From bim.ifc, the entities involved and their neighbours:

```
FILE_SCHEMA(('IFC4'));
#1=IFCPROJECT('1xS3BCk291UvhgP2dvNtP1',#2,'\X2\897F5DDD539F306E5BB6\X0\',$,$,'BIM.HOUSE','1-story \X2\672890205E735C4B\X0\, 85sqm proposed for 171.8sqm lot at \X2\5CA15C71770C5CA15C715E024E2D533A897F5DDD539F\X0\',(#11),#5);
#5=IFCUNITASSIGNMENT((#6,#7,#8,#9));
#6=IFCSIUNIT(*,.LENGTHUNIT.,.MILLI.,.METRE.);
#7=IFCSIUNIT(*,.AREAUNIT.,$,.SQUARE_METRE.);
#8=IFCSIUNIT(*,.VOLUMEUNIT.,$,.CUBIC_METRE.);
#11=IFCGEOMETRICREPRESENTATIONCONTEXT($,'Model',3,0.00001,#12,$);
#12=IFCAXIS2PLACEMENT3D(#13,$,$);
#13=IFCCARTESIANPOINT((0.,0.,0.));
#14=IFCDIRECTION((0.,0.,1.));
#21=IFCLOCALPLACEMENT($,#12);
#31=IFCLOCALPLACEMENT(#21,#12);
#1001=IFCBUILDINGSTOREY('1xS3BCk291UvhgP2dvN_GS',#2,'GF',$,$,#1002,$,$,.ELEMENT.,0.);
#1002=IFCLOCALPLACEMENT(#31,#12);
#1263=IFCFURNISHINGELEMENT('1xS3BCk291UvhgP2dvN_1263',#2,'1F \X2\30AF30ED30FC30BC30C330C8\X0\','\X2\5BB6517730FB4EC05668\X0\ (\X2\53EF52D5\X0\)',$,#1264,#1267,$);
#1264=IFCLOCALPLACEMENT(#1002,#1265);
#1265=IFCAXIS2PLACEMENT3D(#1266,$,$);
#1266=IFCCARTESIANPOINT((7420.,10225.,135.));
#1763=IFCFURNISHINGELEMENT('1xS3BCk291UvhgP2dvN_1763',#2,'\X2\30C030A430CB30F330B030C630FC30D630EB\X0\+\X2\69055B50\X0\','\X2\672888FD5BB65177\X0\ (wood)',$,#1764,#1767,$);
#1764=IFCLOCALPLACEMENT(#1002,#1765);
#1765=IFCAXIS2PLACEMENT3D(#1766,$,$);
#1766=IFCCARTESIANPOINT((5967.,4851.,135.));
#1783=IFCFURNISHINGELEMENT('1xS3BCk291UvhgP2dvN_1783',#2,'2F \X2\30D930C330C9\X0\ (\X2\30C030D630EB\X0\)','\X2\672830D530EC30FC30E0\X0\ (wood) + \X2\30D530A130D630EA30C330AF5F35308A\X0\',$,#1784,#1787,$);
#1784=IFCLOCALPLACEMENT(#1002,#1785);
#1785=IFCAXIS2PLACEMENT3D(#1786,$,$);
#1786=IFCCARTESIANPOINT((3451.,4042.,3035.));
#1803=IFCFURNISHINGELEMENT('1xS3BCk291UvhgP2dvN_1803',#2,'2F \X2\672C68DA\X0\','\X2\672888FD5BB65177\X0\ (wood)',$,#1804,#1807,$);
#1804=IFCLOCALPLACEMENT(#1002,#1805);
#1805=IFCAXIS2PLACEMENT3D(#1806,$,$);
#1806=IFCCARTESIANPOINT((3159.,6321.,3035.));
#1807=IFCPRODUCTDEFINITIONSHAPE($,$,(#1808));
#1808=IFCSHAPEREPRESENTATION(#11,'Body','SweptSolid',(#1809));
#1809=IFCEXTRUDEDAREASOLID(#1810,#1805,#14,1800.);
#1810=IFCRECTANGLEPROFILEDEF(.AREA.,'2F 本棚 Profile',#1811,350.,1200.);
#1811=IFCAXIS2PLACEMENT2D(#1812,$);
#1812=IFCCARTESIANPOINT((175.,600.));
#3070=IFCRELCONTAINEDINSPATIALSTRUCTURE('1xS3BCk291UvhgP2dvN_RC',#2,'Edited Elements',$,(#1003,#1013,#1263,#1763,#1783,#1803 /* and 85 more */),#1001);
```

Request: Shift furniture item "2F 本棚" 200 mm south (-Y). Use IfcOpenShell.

```python
import ifcopenshell
import ifcopenshell.api.geometry
import ifcopenshell.util.placement
import ifcopenshell.util.unit

model = ifcopenshell.open("bim.ifc")
unit_scale = ifcopenshell.util.unit.calculate_unit_scale(model)

item = model.by_guid("1xS3BCk291UvhgP2dvN_1803")
matrix = ifcopenshell.util.placement.get_local_placement(item.ObjectPlacement)
matrix[1, 3] -= 0.2 / unit_scale
ifcopenshell.api.geometry.edit_object_placement(model, product=item, matrix=matrix, is_si=False)

print(ifcopenshell.util.placement.get_local_placement(item.ObjectPlacement).round(3) + 0.0)

model.write("bim_rev.ifc")
```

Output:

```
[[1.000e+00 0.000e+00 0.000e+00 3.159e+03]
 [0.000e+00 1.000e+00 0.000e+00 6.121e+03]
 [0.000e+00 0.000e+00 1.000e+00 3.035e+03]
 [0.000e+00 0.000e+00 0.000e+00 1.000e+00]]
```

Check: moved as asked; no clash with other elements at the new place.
